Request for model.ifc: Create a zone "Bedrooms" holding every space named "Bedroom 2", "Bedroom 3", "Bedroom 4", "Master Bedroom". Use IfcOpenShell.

First a look at what the model holds.

```python
import ifcopenshell

model = ifcopenshell.open("model.ifc")
print(model.schema)
seen = {}
for space in model.by_type("IfcSpace"):
    seen[space.LongName] = seen.get(space.LongName, 0) + 1
for name, count in sorted(seen.items(), key=str):
    print(count, "x", name)
print("zones:", [z.Name for z in model.by_type("IfcZone")][:20])
```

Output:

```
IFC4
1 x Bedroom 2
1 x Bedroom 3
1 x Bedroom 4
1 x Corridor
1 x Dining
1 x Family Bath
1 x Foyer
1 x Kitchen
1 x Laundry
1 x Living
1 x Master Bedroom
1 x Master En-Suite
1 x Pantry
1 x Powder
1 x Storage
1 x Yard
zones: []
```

```python
import ifcopenshell
import ifcopenshell.api.group
import ifcopenshell.api.root

model = ifcopenshell.open("model.ifc")

names = {"Bedroom 2", "Bedroom 3", "Bedroom 4", "Master Bedroom"}
spaces = [s for s in model.by_type("IfcSpace") if s.LongName in names]

zone = ifcopenshell.api.root.create_entity(model, ifc_class="IfcZone", name="Bedrooms")
ifcopenshell.api.group.assign_group(model, products=spaces, group=zone)
print(len(spaces), "spaces in", zone.Name)

model.write("model-out.ifc")
```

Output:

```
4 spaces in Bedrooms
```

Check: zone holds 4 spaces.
